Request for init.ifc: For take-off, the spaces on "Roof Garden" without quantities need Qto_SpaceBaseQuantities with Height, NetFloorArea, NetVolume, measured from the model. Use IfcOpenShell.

First a look at what the model holds.

```python
import ifcopenshell
import ifcopenshell.util.element
import ifcopenshell.util.unit

model = ifcopenshell.open("init.ifc")
print(model.schema)
for unit_type in ("LENGTHUNIT", "AREAUNIT", "VOLUMEUNIT"):
    print(unit_type, ifcopenshell.util.unit.calculate_unit_scale(model, unit_type))
storey = next(s for s in model.by_type("IfcBuildingStorey") if s.Name == "Roof Garden")
spaces = [e for e in ifcopenshell.util.element.get_decomposition(storey) if e.is_a("IfcSpace")]
for e in sorted(spaces, key=lambda e: e.id()):
    print(e.id(), e.is_a(), e.Name, list(ifcopenshell.util.element.get_psets(e, qtos_only=True)), sep=" | ")
```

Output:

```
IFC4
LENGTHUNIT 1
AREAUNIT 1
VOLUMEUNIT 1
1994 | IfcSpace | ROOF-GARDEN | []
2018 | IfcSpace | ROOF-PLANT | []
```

```python
import ifcopenshell
import ifcopenshell.api.pset
import ifcopenshell.geom
import ifcopenshell.util.element
import ifcopenshell.util.shape
import ifcopenshell.util.unit

model = ifcopenshell.open("init.ifc")
unit_scale = ifcopenshell.util.unit.calculate_unit_scale(model)
area_scale = ifcopenshell.util.unit.calculate_unit_scale(model, "AREAUNIT")
volume_scale = ifcopenshell.util.unit.calculate_unit_scale(model, "VOLUMEUNIT")
settings = ifcopenshell.geom.settings()

storey = next(s for s in model.by_type("IfcBuildingStorey") if s.Name == "Roof Garden")
spaces = [e for e in ifcopenshell.util.element.get_decomposition(storey) if e.is_a("IfcSpace")]

for e in sorted(spaces, key=lambda e: e.id()):
    if ifcopenshell.util.element.get_psets(e, qtos_only=True, should_inherit=False):
        continue
    # Geometry comes back in metres, in the element's own axes.
    shape = ifcopenshell.geom.create_shape(settings, e)
    values = {
        "Height": ifcopenshell.util.shape.get_z(shape.geometry) / unit_scale,
        "NetFloorArea": ifcopenshell.util.shape.get_footprint_area(shape.geometry) / area_scale,
        "NetVolume": ifcopenshell.util.shape.get_volume(shape.geometry) / volume_scale,
    }
    qto = ifcopenshell.api.pset.add_qto(model, product=e, name="Qto_SpaceBaseQuantities")
    ifcopenshell.api.pset.edit_qto(model, qto=qto, properties=values)
    print(e.id(), {k: round(v, 3) for k, v in values.items()})

model.write("init-out.ifc")
```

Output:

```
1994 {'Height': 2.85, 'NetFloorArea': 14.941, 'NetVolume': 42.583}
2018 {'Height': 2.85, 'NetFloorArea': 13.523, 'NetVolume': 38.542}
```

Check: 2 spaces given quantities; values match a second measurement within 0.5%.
